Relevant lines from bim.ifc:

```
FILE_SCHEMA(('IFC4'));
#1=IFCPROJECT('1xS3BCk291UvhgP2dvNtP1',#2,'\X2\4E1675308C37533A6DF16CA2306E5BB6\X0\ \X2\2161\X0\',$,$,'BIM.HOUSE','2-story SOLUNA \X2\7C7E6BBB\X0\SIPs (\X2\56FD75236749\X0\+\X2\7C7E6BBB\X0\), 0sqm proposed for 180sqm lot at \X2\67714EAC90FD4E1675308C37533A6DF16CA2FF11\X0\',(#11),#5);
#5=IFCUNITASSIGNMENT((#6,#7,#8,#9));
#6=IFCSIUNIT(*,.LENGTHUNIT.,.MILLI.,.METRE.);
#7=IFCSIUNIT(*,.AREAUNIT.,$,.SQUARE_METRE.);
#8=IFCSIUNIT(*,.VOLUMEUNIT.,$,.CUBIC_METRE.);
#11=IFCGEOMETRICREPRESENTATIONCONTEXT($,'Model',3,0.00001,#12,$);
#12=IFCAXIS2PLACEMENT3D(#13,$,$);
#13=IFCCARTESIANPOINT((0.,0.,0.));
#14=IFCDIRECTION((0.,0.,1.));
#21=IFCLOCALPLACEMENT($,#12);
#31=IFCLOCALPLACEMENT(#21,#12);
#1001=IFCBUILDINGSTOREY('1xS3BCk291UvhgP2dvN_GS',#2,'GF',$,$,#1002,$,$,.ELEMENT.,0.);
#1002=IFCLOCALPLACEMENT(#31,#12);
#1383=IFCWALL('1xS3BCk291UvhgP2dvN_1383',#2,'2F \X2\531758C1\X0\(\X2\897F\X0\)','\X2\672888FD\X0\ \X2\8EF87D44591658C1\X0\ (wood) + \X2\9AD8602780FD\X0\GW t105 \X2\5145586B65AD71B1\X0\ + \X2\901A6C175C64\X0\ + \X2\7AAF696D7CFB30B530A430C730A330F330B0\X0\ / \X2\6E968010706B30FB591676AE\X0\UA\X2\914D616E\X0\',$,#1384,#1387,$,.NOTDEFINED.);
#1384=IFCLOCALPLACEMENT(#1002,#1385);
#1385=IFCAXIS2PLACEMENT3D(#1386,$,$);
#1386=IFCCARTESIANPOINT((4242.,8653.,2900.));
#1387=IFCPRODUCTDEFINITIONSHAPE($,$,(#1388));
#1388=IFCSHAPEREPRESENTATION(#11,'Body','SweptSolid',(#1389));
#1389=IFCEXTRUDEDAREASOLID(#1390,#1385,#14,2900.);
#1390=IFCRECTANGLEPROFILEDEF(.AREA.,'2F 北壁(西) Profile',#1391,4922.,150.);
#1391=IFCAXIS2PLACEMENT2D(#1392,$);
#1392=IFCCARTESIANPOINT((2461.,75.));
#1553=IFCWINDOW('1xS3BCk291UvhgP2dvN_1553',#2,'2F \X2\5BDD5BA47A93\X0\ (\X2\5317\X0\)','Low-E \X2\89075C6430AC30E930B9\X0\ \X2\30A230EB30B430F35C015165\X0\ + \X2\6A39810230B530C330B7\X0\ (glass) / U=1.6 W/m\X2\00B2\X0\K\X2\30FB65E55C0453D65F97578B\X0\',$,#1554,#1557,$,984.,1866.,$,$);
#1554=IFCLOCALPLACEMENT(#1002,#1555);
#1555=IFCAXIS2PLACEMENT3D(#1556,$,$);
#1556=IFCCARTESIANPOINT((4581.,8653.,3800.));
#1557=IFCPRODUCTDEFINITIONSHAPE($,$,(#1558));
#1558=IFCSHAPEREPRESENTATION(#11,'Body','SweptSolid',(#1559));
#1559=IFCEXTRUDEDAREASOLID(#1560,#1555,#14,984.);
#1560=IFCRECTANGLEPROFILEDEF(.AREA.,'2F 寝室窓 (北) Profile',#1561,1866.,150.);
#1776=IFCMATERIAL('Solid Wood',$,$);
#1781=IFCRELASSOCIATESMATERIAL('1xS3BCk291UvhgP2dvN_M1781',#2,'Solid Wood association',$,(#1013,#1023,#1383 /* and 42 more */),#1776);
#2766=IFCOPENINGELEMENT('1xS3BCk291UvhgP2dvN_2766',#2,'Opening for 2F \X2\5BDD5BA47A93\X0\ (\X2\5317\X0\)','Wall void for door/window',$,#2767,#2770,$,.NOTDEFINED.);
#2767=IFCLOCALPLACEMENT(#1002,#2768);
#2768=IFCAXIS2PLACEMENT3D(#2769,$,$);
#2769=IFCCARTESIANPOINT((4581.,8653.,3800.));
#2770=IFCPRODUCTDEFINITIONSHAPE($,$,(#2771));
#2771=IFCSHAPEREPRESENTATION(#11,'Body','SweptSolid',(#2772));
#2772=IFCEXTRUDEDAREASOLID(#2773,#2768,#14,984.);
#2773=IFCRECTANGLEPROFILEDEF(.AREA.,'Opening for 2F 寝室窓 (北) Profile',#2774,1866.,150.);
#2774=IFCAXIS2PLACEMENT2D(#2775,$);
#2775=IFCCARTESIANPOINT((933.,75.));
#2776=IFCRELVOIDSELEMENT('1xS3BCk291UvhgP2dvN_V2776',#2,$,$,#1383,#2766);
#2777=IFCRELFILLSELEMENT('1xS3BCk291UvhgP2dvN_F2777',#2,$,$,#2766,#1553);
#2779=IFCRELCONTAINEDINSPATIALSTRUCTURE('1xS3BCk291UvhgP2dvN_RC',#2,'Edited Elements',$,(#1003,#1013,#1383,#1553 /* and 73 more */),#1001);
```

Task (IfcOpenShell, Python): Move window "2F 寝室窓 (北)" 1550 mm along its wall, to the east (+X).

```python
import ifcopenshell
import ifcopenshell.api.geometry
import ifcopenshell.util.placement
import ifcopenshell.util.unit

model = ifcopenshell.open("bim.ifc")
unit_scale = ifcopenshell.util.unit.calculate_unit_scale(model)

window = model.by_guid("1xS3BCk291UvhgP2dvN_1553")
opening = window.FillsVoids[0].RelatingOpeningElement
wall = opening.VoidsElements[0].RelatingBuildingElement

wall_matrix = ifcopenshell.util.placement.get_local_placement(wall.ObjectPlacement)
shift = wall_matrix[:3, 0] * 1.55 / unit_scale
before = ifcopenshell.util.placement.get_local_placement(window.ObjectPlacement)[:3, 3].copy()

# The window is not placed relative to its opening, so move both.
for product in (opening, window):
    matrix = ifcopenshell.util.placement.get_local_placement(product.ObjectPlacement)
    matrix[:3, 3] += shift
    ifcopenshell.api.geometry.edit_object_placement(model, product=product, matrix=matrix, is_si=False)

after = ifcopenshell.util.placement.get_local_placement(window.ObjectPlacement)[:3, 3]
print("window moved by", (after - before).round(3) + 0.0)

model.write("bim_rev.ifc")
```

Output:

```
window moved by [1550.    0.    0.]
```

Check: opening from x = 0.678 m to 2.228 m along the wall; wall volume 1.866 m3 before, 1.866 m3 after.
